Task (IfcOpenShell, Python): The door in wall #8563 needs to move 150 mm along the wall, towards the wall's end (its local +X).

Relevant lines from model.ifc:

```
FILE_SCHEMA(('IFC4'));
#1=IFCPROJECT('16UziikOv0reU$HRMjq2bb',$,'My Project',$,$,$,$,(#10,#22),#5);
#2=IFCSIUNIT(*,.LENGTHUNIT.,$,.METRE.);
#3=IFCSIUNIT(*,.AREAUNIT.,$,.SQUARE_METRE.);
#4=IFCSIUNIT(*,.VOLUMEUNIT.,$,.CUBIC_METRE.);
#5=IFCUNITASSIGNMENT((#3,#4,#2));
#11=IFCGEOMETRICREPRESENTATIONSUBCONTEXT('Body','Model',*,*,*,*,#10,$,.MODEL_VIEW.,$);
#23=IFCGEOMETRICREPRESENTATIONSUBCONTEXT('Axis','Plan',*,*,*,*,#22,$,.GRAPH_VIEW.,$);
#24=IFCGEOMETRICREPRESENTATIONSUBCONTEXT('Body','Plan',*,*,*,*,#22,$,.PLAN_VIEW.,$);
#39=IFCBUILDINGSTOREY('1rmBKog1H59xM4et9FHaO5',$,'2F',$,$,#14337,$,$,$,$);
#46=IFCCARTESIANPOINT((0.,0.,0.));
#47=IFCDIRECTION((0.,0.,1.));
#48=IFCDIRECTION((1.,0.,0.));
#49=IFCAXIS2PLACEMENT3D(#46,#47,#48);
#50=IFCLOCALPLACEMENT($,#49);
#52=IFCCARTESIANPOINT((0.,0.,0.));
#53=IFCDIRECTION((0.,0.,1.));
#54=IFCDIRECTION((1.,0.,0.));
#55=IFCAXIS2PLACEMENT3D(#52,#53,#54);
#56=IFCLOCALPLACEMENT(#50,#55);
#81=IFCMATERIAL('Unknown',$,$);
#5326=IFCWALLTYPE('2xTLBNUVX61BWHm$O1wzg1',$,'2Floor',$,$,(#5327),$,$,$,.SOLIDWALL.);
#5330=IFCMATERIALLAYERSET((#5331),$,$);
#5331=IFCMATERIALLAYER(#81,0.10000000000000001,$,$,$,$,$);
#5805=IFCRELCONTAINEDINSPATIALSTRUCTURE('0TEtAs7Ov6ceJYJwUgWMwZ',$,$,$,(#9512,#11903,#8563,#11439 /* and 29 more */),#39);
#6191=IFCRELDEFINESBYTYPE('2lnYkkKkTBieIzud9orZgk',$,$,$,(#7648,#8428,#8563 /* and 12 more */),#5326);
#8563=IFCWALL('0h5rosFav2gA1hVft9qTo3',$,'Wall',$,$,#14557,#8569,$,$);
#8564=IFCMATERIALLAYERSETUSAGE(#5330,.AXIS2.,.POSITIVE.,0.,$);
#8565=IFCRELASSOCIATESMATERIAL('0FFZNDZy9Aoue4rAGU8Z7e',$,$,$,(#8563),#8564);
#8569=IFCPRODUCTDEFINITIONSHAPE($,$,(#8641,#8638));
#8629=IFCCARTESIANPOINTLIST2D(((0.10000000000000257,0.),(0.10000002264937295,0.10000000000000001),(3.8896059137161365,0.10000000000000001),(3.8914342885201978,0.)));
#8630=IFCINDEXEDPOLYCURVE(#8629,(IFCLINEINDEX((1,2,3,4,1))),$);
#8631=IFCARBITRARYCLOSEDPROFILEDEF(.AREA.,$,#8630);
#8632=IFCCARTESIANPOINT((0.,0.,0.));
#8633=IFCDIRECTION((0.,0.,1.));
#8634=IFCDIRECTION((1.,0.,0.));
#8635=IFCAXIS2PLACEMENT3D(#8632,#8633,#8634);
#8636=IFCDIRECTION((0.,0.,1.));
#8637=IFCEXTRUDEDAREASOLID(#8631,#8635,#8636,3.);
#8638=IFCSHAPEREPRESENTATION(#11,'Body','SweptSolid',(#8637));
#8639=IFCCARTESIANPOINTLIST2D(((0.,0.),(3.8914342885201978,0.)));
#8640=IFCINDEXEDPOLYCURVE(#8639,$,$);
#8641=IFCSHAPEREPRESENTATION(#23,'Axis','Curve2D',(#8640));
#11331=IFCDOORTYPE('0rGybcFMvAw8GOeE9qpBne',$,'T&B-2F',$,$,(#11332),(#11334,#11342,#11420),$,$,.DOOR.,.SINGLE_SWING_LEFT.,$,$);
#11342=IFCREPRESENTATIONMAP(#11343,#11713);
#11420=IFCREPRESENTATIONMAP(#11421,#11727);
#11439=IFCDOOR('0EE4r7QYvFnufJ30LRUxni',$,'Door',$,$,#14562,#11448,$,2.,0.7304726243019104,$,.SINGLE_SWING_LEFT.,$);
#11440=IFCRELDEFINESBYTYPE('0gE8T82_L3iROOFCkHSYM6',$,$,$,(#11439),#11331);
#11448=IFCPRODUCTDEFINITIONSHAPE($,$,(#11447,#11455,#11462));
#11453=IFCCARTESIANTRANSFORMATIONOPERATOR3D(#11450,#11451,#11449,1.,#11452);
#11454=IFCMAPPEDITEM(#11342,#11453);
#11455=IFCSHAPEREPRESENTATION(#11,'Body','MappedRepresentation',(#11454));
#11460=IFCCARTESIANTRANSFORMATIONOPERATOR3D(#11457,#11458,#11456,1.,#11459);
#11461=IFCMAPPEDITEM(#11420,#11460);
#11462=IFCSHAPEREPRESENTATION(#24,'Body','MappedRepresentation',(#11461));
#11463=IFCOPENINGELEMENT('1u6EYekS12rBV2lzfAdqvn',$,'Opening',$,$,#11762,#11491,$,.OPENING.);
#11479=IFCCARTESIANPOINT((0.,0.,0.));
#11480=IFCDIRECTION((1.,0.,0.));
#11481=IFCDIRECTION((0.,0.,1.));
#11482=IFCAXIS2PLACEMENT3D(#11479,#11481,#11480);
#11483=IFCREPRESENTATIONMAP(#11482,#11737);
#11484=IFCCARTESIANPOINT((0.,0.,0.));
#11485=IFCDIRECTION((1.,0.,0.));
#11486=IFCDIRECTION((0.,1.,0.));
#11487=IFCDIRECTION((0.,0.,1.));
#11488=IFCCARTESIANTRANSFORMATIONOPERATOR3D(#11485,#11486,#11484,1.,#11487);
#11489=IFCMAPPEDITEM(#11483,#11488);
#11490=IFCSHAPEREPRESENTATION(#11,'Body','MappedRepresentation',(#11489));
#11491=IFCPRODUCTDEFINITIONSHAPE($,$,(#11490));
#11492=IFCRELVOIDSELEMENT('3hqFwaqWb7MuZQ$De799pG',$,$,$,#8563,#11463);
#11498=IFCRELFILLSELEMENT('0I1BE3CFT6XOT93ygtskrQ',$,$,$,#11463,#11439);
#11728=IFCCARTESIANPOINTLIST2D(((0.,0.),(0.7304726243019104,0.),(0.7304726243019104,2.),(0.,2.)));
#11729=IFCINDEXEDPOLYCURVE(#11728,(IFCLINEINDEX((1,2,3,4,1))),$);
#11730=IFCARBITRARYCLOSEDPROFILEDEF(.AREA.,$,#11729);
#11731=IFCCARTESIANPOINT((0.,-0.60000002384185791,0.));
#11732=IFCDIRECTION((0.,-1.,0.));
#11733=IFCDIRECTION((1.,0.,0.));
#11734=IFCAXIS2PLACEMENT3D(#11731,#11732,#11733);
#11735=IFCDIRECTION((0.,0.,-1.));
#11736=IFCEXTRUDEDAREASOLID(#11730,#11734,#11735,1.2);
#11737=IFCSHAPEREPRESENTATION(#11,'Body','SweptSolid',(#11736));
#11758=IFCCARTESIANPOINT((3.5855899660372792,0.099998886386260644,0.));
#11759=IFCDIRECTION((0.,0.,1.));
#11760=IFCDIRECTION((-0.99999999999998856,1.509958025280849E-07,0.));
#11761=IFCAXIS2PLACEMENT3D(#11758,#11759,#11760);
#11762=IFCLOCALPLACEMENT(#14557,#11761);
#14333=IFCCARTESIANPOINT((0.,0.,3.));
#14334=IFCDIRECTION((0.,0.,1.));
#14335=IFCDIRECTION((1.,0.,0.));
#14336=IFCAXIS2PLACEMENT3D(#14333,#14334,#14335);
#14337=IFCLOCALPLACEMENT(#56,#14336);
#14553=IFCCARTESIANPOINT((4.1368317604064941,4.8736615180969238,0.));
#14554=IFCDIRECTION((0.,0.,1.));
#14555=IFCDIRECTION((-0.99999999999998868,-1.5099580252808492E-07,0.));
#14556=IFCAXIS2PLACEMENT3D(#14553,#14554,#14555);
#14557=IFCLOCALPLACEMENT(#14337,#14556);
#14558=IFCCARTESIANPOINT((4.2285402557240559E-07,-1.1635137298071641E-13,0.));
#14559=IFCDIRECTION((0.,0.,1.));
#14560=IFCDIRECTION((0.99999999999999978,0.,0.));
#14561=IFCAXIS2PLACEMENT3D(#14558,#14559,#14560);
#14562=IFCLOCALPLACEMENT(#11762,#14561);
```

```python
import ifcopenshell
import ifcopenshell.api.geometry
import ifcopenshell.util.placement

model = ifcopenshell.open("model.ifc")

door = model.by_id(11439)
opening = door.FillsVoids[0].RelatingOpeningElement
wall = opening.VoidsElements[0].RelatingBuildingElement

wall_matrix = ifcopenshell.util.placement.get_local_placement(wall.ObjectPlacement)
shift = wall_matrix[:3, 0] * 0.15
before = ifcopenshell.util.placement.get_local_placement(door.ObjectPlacement)[:3, 3].copy()

# The door is placed relative to its opening, so it follows when the opening moves.
matrix = ifcopenshell.util.placement.get_local_placement(opening.ObjectPlacement)
matrix[:3, 3] += shift
ifcopenshell.api.geometry.edit_object_placement(
    model, product=opening, matrix=matrix, is_si=False, should_transform_children=True
)

after = ifcopenshell.util.placement.get_local_placement(door.ObjectPlacement)[:3, 3]
print("door moved by", (after - before).round(3) + 0.0)

model.write("model-out.ifc")
```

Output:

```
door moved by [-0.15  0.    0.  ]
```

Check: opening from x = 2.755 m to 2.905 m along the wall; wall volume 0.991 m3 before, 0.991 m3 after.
